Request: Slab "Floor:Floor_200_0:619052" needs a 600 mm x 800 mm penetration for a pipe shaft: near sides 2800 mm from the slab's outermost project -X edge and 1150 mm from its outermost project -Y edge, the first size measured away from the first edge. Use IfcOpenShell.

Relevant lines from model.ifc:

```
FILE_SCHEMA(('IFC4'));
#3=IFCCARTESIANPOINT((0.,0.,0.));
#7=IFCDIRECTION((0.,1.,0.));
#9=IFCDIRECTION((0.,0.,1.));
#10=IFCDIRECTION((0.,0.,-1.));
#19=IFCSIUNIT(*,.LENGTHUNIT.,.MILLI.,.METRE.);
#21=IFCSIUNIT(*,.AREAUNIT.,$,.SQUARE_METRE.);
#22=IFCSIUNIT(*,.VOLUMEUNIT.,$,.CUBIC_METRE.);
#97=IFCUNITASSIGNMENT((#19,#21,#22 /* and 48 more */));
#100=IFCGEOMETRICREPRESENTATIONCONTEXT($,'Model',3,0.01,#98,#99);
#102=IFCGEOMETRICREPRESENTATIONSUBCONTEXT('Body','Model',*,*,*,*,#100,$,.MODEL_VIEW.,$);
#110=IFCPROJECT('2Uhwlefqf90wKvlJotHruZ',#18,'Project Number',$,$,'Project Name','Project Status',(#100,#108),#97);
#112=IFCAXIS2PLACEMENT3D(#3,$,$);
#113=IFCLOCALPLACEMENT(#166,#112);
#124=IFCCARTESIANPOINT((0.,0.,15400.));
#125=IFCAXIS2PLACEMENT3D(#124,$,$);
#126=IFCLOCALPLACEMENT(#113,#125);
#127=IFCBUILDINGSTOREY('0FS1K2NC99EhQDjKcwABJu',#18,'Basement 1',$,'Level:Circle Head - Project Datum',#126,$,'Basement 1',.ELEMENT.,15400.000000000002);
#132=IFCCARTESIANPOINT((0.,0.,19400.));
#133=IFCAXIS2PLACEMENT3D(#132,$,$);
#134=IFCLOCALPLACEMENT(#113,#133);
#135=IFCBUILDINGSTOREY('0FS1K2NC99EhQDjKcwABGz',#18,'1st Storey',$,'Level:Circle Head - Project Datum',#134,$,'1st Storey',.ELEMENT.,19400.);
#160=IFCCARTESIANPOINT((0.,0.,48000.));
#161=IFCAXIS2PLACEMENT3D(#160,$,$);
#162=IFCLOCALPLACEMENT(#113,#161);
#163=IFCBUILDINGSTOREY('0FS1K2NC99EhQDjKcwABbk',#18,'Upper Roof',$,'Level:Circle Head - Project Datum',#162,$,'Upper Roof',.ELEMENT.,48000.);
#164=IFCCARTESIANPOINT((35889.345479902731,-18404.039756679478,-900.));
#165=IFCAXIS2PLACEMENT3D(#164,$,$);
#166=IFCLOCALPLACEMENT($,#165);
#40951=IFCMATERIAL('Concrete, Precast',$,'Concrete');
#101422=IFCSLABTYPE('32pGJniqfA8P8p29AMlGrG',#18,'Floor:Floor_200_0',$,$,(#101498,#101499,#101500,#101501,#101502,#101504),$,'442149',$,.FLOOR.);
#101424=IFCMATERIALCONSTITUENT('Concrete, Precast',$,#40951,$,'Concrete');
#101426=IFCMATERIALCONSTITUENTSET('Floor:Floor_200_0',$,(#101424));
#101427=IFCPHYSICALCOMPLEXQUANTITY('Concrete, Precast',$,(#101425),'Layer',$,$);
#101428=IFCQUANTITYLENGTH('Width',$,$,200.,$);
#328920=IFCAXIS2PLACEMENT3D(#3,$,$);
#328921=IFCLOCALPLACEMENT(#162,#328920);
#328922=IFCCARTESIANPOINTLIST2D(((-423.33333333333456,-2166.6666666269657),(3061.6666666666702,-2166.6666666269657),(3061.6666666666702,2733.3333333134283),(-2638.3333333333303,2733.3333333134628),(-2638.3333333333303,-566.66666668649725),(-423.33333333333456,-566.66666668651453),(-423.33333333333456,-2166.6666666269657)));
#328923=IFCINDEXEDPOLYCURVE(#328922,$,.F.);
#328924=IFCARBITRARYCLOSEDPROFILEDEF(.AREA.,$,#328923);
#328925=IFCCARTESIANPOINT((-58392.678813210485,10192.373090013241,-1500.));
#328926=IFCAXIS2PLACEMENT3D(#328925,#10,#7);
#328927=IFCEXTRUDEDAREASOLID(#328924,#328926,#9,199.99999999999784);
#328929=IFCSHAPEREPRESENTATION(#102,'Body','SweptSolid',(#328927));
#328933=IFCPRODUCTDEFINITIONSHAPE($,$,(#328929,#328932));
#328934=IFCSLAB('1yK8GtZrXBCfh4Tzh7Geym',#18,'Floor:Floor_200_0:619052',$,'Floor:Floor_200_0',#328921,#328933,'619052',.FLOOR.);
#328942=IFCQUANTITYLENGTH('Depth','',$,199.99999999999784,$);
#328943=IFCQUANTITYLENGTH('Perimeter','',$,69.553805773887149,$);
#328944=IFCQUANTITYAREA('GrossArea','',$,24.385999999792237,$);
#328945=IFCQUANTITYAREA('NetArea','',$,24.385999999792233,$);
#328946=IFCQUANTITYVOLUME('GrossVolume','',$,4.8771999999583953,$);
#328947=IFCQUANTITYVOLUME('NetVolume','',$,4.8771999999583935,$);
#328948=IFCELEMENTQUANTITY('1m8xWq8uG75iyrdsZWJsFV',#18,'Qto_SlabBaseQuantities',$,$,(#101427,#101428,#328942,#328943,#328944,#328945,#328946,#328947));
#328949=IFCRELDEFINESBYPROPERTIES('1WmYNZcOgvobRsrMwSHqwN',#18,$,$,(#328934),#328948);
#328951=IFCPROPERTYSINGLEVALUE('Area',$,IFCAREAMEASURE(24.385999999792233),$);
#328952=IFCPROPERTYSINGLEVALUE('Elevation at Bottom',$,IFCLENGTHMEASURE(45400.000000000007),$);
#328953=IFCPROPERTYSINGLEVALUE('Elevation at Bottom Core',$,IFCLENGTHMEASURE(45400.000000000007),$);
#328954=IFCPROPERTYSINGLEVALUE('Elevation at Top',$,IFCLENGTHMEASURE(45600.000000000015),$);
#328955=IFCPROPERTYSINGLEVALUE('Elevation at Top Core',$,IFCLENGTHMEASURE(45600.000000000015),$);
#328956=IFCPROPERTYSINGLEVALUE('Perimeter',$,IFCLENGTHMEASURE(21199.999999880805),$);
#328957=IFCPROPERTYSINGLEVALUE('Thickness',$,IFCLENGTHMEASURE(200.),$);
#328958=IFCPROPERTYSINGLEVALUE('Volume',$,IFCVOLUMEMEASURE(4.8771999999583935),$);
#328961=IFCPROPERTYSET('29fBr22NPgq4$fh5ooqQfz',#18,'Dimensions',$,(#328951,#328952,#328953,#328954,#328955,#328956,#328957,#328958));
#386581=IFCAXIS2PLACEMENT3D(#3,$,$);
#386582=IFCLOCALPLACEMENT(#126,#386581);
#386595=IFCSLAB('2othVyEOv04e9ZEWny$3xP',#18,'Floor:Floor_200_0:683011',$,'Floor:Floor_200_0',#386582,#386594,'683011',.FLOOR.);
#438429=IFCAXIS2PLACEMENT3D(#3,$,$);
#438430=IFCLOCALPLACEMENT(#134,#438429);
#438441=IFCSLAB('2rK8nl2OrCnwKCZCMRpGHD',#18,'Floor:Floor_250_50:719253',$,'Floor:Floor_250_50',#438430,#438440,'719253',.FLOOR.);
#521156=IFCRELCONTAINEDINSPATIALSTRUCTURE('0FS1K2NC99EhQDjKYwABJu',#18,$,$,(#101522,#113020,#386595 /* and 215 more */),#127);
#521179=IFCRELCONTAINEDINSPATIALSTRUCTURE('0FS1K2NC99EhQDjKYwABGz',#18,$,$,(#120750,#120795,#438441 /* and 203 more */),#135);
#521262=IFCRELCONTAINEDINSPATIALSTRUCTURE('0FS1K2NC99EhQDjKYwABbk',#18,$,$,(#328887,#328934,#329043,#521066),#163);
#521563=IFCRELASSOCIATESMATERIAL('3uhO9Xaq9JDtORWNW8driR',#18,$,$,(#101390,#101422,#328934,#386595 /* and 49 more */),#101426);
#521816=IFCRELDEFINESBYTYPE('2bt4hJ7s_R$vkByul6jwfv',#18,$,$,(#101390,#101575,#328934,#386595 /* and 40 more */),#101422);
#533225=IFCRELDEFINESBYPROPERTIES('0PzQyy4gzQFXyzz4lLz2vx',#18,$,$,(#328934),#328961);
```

```python
import numpy as np
import ifcopenshell
import ifcopenshell.api.feature
import ifcopenshell.api.geometry
import ifcopenshell.api.pset
import ifcopenshell.api.root
import ifcopenshell.geom
import ifcopenshell.util.element
import ifcopenshell.util.placement
import ifcopenshell.util.representation
import ifcopenshell.util.shape
import ifcopenshell.util.unit

model = ifcopenshell.open("model.ifc")
unit_scale = ifcopenshell.util.unit.calculate_unit_scale(model)
area_scale = ifcopenshell.util.unit.calculate_unit_scale(model, "AREAUNIT")
volume_scale = ifcopenshell.util.unit.calculate_unit_scale(model, "VOLUMEUNIT")
settings = ifcopenshell.geom.settings()


def volume(element):
    """Net volume in cubic metres, openings subtracted."""
    shape = ifcopenshell.geom.create_shape(settings, element)
    return ifcopenshell.util.shape.get_volume(shape.geometry)


slab = model.by_guid("1yK8GtZrXBCfh4Tzh7Geym")
before = volume(slab)

# Extent in the slab's own axes, in metres. The edges named are its -X and -Y sides.
slab_shape = ifcopenshell.geom.create_shape(settings, slab)
vertices = ifcopenshell.util.shape.get_vertices(slab_shape.geometry)
x_min, y_min, bottom = vertices.min(axis=0)
top = vertices[:, 2].max()

opening = ifcopenshell.api.root.create_entity(model, ifc_class="IfcOpeningElement", name="Pipe shaft opening", predefined_type="OPENING")
context = ifcopenshell.util.representation.get_context(model, "Model", "Body", "MODEL_VIEW")
width, depth = 0.6, 0.8
outline = [(0.0, 0.0), (width, 0.0), (width, depth), (0.0, depth), (0.0, 0.0)]
# Overshoot both faces by 50 mm so the cut is clean.
shape = ifcopenshell.api.geometry.add_slab_representation(
    model, context=context, depth=top - bottom + 0.1, polyline=outline
)
ifcopenshell.api.geometry.assign_representation(model, product=opening, representation=shape)

matrix = ifcopenshell.util.placement.get_local_placement(slab.ObjectPlacement)
matrix[:, 3] = matrix @ np.append(np.array([x_min + 2.8, y_min + 1.15, bottom - 0.05]) / unit_scale, 1.0)
ifcopenshell.api.geometry.edit_object_placement(model, product=opening, matrix=matrix, is_si=False)
ifcopenshell.api.feature.add_feature(model, feature=opening, element=slab)

after = volume(slab)

# Update the slab's stored quantities.
qto = model.by_id(ifcopenshell.util.element.get_pset(slab, "Qto_SlabBaseQuantities", should_inherit=False)["id"])
ifcopenshell.api.pset.edit_qto(model, qto=qto, properties={
    "NetArea": after / (top - bottom) / area_scale,
    "NetVolume": after / volume_scale,
})
pset = model.by_id(ifcopenshell.util.element.get_pset(slab, "Dimensions", should_inherit=False)["id"])
ifcopenshell.api.pset.edit_pset(model, pset=pset, properties={
    "Area": model.create_entity("IfcAreaMeasure", after / (top - bottom) / area_scale),
    "Volume": model.create_entity("IfcVolumeMeasure", after / volume_scale),
})

print(f"slab volume {before:.3f} -> {after:.3f} m3")

model.write("model_updated.ifc")
```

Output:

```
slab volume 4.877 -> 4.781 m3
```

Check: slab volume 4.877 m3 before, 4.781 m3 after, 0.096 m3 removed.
